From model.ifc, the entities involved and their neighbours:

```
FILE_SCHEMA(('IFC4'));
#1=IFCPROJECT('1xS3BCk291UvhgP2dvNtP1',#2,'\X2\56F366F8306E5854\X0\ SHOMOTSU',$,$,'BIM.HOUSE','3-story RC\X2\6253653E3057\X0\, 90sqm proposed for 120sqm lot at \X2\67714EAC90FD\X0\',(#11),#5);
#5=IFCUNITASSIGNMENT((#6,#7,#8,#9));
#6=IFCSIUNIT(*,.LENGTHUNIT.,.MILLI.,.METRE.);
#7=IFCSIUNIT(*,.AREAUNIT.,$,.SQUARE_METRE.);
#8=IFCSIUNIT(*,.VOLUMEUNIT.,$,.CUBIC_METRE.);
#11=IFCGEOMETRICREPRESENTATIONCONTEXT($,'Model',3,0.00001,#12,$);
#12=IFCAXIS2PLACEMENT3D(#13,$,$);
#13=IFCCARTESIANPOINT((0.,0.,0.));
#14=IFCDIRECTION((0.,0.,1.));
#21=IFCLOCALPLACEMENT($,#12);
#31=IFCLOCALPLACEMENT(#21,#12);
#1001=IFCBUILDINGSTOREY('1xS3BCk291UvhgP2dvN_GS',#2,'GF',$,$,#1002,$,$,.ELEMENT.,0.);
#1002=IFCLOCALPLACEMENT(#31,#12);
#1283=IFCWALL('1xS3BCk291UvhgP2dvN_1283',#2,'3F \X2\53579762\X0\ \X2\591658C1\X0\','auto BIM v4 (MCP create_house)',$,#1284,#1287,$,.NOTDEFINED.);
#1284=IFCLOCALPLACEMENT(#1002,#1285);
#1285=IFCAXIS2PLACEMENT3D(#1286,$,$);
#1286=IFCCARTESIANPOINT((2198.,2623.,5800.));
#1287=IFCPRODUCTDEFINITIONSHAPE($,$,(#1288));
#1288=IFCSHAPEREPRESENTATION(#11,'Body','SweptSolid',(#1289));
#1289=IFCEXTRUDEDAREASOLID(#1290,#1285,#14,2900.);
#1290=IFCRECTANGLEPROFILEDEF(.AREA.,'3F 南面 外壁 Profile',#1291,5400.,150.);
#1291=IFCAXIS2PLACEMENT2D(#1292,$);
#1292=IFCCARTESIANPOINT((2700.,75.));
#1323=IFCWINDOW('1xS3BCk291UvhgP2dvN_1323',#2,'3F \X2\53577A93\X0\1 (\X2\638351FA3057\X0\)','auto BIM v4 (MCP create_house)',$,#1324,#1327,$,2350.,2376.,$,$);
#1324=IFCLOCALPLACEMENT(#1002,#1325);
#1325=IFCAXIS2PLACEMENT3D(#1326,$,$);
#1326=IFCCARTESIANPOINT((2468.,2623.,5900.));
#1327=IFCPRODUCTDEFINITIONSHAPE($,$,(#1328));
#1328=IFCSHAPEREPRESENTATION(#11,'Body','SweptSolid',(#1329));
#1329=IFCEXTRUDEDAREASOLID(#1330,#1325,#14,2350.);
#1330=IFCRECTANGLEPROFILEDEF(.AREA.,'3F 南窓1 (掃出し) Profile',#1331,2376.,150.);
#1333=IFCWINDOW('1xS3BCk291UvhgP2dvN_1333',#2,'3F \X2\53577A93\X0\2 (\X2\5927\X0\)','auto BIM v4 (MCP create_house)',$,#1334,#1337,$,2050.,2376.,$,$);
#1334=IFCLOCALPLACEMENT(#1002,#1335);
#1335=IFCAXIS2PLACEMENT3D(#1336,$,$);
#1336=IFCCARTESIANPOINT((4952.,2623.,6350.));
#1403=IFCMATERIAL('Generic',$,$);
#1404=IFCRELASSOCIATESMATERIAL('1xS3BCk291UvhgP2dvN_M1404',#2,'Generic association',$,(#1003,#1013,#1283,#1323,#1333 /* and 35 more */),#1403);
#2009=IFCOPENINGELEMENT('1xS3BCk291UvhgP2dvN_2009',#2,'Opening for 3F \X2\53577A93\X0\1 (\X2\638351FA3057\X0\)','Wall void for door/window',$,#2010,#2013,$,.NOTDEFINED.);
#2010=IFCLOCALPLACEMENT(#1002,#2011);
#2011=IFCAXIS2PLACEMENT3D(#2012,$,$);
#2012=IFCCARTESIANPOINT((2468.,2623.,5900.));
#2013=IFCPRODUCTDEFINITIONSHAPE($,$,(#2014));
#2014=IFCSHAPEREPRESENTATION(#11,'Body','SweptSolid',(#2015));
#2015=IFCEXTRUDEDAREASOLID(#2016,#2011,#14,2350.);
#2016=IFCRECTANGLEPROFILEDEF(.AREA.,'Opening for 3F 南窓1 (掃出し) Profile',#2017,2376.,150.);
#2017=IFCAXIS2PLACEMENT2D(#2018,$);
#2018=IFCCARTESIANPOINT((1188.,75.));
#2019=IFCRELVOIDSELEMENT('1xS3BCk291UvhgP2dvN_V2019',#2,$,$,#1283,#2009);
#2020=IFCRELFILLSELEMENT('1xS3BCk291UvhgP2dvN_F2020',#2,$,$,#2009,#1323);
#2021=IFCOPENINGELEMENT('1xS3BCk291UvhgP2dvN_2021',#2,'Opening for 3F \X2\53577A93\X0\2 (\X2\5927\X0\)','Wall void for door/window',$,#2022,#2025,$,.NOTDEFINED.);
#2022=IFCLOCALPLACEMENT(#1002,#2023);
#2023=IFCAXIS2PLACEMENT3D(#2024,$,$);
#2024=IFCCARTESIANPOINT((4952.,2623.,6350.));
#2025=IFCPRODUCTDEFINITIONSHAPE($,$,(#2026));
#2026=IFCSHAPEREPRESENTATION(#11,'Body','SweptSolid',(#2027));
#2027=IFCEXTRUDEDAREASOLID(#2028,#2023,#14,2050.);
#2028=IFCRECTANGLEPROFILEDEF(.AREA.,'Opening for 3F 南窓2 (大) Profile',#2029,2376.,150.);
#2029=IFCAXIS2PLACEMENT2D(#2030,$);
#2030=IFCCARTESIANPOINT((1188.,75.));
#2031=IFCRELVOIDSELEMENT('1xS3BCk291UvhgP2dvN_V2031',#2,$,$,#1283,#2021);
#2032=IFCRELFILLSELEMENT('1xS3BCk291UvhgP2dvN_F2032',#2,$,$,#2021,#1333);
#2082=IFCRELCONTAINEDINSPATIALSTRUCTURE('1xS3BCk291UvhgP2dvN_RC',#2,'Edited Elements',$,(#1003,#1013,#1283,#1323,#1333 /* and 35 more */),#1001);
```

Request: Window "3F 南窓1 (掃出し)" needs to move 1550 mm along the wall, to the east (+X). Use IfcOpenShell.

```python
import ifcopenshell
import ifcopenshell.api.geometry
import ifcopenshell.util.placement
import ifcopenshell.util.unit

model = ifcopenshell.open("model.ifc")
unit_scale = ifcopenshell.util.unit.calculate_unit_scale(model)

window = model.by_guid("1xS3BCk291UvhgP2dvN_1323")
opening = window.FillsVoids[0].RelatingOpeningElement
wall = opening.VoidsElements[0].RelatingBuildingElement

wall_matrix = ifcopenshell.util.placement.get_local_placement(wall.ObjectPlacement)
shift = wall_matrix[:3, 0] * 1.55 / unit_scale
before = ifcopenshell.util.placement.get_local_placement(window.ObjectPlacement)[:3, 3].copy()

# The window is not placed relative to its opening, so move both.
for product in (opening, window):
    matrix = ifcopenshell.util.placement.get_local_placement(product.ObjectPlacement)
    matrix[:3, 3] += shift
    ifcopenshell.api.geometry.edit_object_placement(model, product=product, matrix=matrix, is_si=False)

after = ifcopenshell.util.placement.get_local_placement(window.ObjectPlacement)[:3, 3]
print("window moved by", (after - before).round(3) + 0.0)

model.write("model_edited.ifc")
```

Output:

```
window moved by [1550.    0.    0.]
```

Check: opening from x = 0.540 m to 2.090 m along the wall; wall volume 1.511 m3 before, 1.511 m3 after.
